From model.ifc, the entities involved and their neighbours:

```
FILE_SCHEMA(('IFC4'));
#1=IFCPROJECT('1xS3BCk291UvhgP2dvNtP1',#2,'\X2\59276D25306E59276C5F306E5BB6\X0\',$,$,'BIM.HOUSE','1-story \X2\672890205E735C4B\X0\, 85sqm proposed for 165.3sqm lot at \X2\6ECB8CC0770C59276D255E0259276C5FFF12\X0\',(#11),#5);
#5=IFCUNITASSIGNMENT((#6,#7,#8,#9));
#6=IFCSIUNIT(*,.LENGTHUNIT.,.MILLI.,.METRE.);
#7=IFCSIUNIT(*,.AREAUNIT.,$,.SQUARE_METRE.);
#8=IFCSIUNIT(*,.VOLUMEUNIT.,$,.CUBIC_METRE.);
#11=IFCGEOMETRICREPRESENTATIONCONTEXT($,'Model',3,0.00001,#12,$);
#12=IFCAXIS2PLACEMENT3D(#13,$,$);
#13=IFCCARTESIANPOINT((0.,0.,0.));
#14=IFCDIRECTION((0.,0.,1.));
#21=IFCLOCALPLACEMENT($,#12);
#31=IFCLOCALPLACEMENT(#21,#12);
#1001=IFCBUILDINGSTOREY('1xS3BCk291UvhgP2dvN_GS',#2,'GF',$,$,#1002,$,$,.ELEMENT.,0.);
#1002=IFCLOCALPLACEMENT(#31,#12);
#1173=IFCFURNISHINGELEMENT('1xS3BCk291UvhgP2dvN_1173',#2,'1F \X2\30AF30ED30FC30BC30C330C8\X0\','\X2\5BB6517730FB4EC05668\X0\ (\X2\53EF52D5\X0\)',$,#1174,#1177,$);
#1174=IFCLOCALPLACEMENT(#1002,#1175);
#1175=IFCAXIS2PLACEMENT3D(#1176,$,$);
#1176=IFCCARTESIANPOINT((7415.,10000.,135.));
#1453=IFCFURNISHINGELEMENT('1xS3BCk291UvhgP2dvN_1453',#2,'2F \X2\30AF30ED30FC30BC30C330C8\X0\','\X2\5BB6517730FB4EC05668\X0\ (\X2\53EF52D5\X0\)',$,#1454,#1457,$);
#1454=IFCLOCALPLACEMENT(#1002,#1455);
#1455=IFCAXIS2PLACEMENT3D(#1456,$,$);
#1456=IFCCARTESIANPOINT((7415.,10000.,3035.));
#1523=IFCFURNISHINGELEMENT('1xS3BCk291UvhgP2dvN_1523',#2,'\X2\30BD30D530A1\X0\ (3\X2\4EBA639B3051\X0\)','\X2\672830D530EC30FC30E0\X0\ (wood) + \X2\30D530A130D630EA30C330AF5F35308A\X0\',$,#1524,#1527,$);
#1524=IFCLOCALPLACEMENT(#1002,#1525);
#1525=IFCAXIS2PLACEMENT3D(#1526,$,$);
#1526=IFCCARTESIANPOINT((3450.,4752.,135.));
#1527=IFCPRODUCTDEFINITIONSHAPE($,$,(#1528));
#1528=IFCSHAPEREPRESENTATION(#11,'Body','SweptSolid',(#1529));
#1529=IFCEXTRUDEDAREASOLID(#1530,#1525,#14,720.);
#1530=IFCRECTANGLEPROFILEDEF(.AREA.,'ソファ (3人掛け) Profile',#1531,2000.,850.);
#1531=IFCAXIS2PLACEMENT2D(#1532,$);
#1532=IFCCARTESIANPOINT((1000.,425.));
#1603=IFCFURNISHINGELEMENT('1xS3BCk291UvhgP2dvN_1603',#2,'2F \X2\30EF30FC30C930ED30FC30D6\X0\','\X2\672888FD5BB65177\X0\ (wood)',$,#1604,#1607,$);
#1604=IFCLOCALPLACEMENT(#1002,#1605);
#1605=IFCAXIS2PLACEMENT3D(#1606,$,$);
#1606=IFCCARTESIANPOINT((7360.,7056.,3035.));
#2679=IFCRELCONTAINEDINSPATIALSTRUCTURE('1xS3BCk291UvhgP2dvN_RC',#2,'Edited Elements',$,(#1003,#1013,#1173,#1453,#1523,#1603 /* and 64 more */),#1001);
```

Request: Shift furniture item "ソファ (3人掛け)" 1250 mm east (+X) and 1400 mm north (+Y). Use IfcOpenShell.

```python
import ifcopenshell
import ifcopenshell.api.geometry
import ifcopenshell.util.placement
import ifcopenshell.util.unit

model = ifcopenshell.open("model.ifc")
unit_scale = ifcopenshell.util.unit.calculate_unit_scale(model)

item = model.by_id(1523)
matrix = ifcopenshell.util.placement.get_local_placement(item.ObjectPlacement)
matrix[0, 3] += 1.25 / unit_scale
matrix[1, 3] += 1.4 / unit_scale
ifcopenshell.api.geometry.edit_object_placement(model, product=item, matrix=matrix, is_si=False)

print(ifcopenshell.util.placement.get_local_placement(item.ObjectPlacement).round(3) + 0.0)

model.write("model_edited.ifc")
```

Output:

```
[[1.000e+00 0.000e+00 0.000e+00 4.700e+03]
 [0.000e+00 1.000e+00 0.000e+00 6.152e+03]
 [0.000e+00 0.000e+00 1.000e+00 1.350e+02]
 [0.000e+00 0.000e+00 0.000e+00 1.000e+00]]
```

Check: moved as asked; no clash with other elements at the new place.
